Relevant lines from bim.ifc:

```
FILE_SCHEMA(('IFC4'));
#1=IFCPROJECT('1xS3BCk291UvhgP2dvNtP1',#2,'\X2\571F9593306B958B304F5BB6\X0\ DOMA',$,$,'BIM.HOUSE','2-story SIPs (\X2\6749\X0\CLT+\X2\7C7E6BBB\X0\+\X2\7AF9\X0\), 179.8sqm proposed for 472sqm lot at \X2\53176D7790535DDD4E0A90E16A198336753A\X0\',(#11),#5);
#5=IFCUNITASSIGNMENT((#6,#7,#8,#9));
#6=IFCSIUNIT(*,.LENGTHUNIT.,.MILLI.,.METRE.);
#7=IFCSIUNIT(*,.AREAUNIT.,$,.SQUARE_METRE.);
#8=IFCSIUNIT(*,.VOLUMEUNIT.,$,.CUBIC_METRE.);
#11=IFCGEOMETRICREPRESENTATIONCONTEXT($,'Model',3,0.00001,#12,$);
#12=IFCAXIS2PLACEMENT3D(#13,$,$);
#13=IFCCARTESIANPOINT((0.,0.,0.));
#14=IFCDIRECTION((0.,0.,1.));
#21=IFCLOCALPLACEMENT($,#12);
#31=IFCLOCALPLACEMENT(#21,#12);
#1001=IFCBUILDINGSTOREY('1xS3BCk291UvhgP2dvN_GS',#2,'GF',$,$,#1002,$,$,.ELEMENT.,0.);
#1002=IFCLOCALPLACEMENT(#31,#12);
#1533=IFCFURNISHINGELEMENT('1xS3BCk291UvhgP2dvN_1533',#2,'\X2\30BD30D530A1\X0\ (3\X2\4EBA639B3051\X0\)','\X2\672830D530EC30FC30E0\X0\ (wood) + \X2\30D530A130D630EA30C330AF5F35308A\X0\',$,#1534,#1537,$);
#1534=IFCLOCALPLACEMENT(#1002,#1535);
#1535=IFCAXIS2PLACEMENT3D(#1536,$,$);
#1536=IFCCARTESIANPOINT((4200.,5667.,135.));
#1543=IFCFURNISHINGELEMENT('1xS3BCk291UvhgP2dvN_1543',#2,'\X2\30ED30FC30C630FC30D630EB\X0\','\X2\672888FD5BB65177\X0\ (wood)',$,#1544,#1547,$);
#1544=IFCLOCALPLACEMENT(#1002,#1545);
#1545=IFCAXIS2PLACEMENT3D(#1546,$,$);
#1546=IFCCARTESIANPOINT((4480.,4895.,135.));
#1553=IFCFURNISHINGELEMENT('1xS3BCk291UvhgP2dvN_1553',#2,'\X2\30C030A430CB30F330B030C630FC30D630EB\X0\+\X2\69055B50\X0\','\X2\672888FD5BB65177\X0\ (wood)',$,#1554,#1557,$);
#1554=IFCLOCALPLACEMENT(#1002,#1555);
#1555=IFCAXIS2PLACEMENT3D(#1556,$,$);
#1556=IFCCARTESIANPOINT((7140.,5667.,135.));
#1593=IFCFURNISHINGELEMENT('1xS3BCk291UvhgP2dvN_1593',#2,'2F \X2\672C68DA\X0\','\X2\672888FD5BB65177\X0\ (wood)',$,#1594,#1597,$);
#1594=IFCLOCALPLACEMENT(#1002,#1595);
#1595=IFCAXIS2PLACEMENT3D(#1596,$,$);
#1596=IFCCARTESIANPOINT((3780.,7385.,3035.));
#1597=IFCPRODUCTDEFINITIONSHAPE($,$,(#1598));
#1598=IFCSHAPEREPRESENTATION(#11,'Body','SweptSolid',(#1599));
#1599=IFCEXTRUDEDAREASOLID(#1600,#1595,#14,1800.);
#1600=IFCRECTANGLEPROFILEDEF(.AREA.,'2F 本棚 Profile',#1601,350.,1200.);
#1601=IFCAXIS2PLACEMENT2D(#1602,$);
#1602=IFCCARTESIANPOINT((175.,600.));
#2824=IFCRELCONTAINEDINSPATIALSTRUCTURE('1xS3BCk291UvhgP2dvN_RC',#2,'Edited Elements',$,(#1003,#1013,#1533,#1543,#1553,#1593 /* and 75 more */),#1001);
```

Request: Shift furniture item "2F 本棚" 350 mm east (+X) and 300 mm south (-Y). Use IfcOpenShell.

```python
import ifcopenshell
import ifcopenshell.api.geometry
import ifcopenshell.util.placement
import ifcopenshell.util.unit

model = ifcopenshell.open("bim.ifc")
unit_scale = ifcopenshell.util.unit.calculate_unit_scale(model)

item = model.by_guid("1xS3BCk291UvhgP2dvN_1593")
matrix = ifcopenshell.util.placement.get_local_placement(item.ObjectPlacement)
matrix[0, 3] += 0.35 / unit_scale
matrix[1, 3] -= 0.3 / unit_scale
ifcopenshell.api.geometry.edit_object_placement(model, product=item, matrix=matrix, is_si=False)

print(ifcopenshell.util.placement.get_local_placement(item.ObjectPlacement).round(3) + 0.0)

model.write("bim_rev.ifc")
```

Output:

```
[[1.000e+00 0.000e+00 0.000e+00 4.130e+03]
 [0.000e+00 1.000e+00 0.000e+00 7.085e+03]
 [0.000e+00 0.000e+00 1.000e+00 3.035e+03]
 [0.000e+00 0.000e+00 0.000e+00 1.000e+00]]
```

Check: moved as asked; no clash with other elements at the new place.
